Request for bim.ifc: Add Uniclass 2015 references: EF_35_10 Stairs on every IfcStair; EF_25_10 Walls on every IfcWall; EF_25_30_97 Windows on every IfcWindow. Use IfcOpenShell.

First a look at what the model holds.

```python
import ifcopenshell

model = ifcopenshell.open("bim.ifc")
print(model.schema)
print("classifications:", [c.Name for c in model.by_type("IfcClassification")])
for ifc_class in ("IfcDoor", "IfcRoof", "IfcStair", "IfcWall", "IfcWindow"):
    print(ifc_class, len(model.by_type(ifc_class)))
```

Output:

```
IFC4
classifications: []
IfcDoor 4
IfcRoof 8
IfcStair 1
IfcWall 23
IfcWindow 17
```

```python
import ifcopenshell
import ifcopenshell.api.classification

model = ifcopenshell.open("bim.ifc")

system = ifcopenshell.api.classification.add_classification(model, classification="Uniclass 2015")

codes = {
    "IfcStair": ("EF_35_10", "Stairs"),
    "IfcWall": ("EF_25_10", "Walls"),
    "IfcWindow": ("EF_25_30_97", "Windows"),
}
for ifc_class, (code, name) in codes.items():
    products = model.by_type(ifc_class)
    ifcopenshell.api.classification.add_reference(
        model, products=products, classification=system, identification=code, name=name
    )
    print(code, len(products))

model.write("bim_edited.ifc")
```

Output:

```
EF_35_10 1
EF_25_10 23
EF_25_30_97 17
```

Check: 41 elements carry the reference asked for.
